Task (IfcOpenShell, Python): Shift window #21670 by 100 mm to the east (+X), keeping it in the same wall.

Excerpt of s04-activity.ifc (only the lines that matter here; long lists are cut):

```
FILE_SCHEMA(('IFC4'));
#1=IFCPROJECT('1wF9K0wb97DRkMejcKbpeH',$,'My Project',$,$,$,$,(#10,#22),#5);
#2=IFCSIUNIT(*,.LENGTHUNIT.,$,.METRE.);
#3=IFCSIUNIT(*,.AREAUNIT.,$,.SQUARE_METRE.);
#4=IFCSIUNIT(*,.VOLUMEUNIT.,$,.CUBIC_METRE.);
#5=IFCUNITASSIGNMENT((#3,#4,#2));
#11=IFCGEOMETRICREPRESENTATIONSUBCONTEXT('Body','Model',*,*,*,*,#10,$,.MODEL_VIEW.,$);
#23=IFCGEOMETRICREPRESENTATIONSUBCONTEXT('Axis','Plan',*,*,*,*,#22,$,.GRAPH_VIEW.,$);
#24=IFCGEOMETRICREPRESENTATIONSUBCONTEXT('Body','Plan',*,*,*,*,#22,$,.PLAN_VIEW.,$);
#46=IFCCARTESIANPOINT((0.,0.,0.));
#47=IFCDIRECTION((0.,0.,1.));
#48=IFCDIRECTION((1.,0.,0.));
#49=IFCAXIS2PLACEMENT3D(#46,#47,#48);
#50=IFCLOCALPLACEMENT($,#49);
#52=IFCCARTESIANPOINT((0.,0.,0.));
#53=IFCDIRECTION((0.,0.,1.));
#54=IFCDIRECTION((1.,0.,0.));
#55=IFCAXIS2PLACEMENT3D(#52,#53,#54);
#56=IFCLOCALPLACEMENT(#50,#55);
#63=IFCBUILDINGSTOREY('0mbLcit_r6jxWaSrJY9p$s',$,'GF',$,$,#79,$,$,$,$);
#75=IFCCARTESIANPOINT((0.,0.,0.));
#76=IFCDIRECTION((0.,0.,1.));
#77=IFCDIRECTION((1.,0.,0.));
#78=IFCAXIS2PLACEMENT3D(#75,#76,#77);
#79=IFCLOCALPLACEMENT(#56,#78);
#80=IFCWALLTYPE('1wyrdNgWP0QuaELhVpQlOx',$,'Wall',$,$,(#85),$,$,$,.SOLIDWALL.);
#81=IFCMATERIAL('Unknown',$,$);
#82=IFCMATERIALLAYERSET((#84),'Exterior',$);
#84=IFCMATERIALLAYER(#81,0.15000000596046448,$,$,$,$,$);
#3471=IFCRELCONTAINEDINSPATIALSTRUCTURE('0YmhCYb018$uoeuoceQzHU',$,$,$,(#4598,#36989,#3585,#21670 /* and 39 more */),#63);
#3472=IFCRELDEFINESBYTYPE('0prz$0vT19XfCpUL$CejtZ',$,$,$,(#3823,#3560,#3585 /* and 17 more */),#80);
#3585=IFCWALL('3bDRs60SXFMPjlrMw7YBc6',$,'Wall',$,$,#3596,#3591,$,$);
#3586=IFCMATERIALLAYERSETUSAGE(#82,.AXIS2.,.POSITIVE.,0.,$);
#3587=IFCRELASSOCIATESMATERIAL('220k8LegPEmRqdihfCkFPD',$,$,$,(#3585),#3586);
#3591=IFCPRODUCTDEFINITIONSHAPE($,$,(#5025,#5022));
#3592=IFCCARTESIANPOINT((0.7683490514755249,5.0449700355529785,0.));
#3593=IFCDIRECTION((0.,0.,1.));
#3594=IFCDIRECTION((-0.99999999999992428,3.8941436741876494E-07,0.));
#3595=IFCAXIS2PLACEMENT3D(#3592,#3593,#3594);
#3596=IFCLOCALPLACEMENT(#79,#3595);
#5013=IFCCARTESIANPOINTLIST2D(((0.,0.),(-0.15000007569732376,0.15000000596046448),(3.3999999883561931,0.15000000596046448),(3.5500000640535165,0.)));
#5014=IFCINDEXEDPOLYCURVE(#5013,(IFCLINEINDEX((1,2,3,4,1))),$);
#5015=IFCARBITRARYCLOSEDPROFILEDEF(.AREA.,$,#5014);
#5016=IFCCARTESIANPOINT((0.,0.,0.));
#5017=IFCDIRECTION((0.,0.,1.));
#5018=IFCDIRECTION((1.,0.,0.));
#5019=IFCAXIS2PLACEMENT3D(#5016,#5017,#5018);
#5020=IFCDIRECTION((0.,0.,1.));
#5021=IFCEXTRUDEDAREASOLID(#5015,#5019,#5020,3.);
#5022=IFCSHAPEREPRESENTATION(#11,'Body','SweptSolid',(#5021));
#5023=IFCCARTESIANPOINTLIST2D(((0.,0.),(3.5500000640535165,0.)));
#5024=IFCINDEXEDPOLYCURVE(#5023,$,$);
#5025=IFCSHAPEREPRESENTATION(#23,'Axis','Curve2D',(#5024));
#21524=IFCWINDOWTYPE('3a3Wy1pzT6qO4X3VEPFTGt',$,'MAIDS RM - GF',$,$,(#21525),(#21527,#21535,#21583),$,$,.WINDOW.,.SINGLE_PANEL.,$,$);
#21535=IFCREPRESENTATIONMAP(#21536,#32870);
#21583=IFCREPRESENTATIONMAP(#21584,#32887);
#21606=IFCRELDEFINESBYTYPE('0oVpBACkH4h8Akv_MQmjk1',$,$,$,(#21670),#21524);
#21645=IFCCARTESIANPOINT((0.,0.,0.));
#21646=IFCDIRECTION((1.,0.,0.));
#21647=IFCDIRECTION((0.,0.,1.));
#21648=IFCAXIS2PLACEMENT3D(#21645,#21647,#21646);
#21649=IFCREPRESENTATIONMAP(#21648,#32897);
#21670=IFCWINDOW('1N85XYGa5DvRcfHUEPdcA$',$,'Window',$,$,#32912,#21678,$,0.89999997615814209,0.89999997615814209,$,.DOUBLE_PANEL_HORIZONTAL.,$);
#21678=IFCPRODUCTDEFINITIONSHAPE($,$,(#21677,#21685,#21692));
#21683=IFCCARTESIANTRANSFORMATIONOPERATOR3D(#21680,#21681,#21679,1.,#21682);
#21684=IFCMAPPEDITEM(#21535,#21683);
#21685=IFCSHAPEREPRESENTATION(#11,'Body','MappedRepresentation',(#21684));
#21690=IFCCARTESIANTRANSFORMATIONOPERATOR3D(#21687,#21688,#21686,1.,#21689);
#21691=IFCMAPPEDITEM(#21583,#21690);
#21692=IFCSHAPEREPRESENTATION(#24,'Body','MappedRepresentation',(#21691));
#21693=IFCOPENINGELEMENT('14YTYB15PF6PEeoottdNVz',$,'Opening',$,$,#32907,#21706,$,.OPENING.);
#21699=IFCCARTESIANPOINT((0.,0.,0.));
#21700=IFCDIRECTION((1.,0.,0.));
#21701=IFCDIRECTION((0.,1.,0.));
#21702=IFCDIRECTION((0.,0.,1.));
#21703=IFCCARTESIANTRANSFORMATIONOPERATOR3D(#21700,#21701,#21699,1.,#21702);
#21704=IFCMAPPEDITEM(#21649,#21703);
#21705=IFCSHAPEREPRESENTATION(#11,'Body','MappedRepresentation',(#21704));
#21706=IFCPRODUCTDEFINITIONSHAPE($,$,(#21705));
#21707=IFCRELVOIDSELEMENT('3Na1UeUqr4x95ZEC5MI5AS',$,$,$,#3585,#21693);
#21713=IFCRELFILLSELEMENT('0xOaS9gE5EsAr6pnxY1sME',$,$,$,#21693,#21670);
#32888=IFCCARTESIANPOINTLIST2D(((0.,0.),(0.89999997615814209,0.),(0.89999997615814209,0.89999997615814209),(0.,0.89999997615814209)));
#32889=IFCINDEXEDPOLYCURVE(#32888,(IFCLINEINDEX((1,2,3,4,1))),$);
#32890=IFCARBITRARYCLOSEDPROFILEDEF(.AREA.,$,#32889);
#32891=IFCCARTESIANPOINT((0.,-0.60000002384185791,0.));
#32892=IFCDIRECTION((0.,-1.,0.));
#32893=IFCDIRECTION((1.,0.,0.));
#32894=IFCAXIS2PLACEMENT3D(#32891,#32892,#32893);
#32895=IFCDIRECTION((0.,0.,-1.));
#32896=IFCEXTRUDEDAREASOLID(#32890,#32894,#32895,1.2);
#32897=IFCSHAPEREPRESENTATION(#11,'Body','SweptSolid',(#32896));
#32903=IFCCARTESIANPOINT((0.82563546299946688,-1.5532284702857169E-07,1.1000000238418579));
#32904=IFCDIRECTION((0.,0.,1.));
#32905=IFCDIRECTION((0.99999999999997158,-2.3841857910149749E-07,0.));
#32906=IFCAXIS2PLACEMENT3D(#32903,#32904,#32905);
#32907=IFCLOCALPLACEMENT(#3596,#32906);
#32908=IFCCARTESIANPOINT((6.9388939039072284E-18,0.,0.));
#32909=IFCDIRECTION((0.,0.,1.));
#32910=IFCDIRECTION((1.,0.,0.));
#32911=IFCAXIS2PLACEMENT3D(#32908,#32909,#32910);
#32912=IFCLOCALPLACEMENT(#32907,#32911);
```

```python
import ifcopenshell
import ifcopenshell.api.geometry
import ifcopenshell.util.placement

model = ifcopenshell.open("s04-activity.ifc")

window = model.by_guid("1N85XYGa5DvRcfHUEPdcA$")
opening = window.FillsVoids[0].RelatingOpeningElement
wall = opening.VoidsElements[0].RelatingBuildingElement

wall_matrix = ifcopenshell.util.placement.get_local_placement(wall.ObjectPlacement)
shift = wall_matrix[:3, 0] * -0.1
before = ifcopenshell.util.placement.get_local_placement(window.ObjectPlacement)[:3, 3].copy()

# The window is placed relative to its opening, so it follows when the opening moves.
matrix = ifcopenshell.util.placement.get_local_placement(opening.ObjectPlacement)
matrix[:3, 3] += shift
ifcopenshell.api.geometry.edit_object_placement(
    model, product=opening, matrix=matrix, is_si=False, should_transform_children=True
)

after = ifcopenshell.util.placement.get_local_placement(window.ObjectPlacement)[:3, 3]
print("window moved by", (after - before).round(3) + 0.0)

model.write("s04-activity_updated.ifc")
```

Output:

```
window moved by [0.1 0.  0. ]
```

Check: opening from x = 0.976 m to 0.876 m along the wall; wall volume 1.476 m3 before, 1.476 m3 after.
